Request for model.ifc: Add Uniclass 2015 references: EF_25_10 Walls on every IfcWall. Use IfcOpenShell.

First a look at what the model holds.

```python
import ifcopenshell

model = ifcopenshell.open("model.ifc")
print(model.schema)
print("classifications:", [c.Name for c in model.by_type("IfcClassification")])
for ifc_class in ("IfcDoor", "IfcRoof", "IfcStair", "IfcWall", "IfcWindow"):
    print(ifc_class, len(model.by_type(ifc_class)))
```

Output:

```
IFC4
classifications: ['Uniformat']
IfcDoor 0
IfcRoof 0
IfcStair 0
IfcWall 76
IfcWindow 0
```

```python
import ifcopenshell
import ifcopenshell.api.classification

model = ifcopenshell.open("model.ifc")

system = ifcopenshell.api.classification.add_classification(model, classification="Uniclass 2015")

codes = {
    "IfcWall": ("EF_25_10", "Walls"),
}
for ifc_class, (code, name) in codes.items():
    products = model.by_type(ifc_class)
    ifcopenshell.api.classification.add_reference(
        model, products=products, classification=system, identification=code, name=name
    )
    print(code, len(products))

model.write("model_edited.ifc")
```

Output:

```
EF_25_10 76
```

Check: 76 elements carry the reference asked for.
